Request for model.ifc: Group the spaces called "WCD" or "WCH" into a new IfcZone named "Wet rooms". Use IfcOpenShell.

First a look at what the model holds.

```python
import ifcopenshell

model = ifcopenshell.open("model.ifc")
print(model.schema)
seen = {}
for space in model.by_type("IfcSpace"):
    seen[space.LongName] = seen.get(space.LongName, 0) + 1
for name, count in sorted(seen.items(), key=str):
    print(count, "x", name)
print("zones:", [z.Name for z in model.by_type("IfcZone")][:20])
```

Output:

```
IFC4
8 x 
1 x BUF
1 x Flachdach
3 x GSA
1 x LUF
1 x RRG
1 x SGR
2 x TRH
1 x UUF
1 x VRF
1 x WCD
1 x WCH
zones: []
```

```python
import ifcopenshell
import ifcopenshell.api.group
import ifcopenshell.api.root

model = ifcopenshell.open("model.ifc")

names = {"WCD", "WCH"}
spaces = [s for s in model.by_type("IfcSpace") if s.LongName in names]

zone = ifcopenshell.api.root.create_entity(model, ifc_class="IfcZone", name="Wet rooms")
ifcopenshell.api.group.assign_group(model, products=spaces, group=zone)
print(len(spaces), "spaces in", zone.Name)

model.write("model_v2.ifc")
```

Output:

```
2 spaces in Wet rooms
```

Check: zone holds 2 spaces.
